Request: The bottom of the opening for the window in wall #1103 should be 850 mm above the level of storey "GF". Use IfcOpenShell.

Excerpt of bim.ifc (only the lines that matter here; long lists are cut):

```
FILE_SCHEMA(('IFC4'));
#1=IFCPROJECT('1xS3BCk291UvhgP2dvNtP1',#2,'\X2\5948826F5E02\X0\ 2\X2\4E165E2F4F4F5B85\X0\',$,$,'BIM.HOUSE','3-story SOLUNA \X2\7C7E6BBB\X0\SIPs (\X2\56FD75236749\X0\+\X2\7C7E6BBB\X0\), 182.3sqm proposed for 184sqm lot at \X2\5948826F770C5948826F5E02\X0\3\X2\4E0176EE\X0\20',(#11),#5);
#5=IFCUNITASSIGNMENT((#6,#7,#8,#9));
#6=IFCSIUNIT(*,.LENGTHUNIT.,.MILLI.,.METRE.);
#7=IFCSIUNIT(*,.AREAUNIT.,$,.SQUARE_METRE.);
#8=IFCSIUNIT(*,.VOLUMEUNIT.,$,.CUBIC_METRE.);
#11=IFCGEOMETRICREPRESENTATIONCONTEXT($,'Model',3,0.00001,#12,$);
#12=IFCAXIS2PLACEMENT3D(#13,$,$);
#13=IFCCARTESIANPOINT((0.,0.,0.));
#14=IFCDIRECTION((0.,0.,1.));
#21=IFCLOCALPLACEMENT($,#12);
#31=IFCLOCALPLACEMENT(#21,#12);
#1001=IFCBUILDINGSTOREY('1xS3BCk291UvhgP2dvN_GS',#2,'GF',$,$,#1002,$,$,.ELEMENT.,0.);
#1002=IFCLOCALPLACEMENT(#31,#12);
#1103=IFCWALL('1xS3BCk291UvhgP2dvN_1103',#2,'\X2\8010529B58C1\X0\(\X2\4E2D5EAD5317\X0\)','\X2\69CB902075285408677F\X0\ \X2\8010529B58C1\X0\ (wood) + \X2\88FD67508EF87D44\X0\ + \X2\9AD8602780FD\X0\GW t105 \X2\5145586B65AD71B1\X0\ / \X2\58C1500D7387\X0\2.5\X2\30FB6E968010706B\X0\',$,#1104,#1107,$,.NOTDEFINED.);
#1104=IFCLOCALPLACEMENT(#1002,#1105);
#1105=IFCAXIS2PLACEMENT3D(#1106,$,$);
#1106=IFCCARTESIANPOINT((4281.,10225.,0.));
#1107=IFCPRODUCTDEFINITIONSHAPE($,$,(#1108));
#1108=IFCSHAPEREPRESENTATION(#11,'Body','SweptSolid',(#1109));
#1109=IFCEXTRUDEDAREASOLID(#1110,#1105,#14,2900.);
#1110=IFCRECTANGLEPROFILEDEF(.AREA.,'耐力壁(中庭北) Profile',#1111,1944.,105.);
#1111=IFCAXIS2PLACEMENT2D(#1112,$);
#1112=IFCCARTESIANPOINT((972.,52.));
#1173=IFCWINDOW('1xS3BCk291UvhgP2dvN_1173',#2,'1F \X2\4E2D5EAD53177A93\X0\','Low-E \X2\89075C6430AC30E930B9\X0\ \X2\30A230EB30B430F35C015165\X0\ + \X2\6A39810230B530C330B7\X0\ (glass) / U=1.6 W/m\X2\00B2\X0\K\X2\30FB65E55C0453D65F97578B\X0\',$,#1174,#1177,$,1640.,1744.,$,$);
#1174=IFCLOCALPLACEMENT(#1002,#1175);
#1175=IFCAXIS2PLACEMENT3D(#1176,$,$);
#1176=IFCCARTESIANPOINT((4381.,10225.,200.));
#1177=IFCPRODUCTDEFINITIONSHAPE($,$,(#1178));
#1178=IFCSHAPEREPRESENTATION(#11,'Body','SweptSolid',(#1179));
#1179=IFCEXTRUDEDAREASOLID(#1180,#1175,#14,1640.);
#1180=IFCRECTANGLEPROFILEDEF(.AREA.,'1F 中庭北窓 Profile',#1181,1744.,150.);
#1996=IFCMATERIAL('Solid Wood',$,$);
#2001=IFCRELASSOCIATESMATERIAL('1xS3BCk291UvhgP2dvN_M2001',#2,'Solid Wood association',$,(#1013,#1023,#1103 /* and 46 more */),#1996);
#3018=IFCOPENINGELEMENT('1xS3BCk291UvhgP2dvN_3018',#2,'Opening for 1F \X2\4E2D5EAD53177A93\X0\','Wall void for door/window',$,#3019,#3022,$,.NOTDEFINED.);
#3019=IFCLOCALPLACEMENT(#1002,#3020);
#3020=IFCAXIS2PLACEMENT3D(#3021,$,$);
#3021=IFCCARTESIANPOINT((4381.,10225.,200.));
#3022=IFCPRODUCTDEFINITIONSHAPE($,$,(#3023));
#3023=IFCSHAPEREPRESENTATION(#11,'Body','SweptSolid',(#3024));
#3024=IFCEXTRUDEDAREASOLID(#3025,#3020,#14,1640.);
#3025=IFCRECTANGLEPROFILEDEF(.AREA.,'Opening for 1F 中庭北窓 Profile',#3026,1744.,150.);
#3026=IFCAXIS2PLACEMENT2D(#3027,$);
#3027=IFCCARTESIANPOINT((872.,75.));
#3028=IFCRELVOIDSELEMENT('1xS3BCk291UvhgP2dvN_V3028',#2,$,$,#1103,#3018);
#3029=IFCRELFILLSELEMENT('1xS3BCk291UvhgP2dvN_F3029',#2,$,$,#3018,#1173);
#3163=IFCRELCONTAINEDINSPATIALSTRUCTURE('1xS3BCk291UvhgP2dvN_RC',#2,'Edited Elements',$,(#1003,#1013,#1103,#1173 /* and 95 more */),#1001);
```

```python
import numpy as np
import ifcopenshell
import ifcopenshell.api.geometry
import ifcopenshell.geom
import ifcopenshell.util.element
import ifcopenshell.util.placement
import ifcopenshell.util.shape
import ifcopenshell.util.unit

model = ifcopenshell.open("bim.ifc")
unit_scale = ifcopenshell.util.unit.calculate_unit_scale(model)

window = model.by_id(1173)
opening = window.FillsVoids[0].RelatingOpeningElement
storey = ifcopenshell.util.element.get_container(window, ifc_class="IfcBuildingStorey")
level = ifcopenshell.util.placement.get_local_placement(storey.ObjectPlacement)[2, 3]

# The opening's origin need not be at the sill, so measure its lowest point.
shape = ifcopenshell.geom.create_shape(ifcopenshell.geom.settings(), opening)
bottom = ifcopenshell.util.shape.get_shape_bottom_elevation(shape, shape.geometry) / unit_scale
dz = level + 850.0 - bottom

shift = np.array([0.0, 0.0, dz])
# The window is not placed relative to its opening, so move both.
for product in (opening, window):
    matrix = ifcopenshell.util.placement.get_local_placement(product.ObjectPlacement)
    matrix[:3, 3] += shift
    ifcopenshell.api.geometry.edit_object_placement(model, product=product, matrix=matrix, is_si=False)

print(f"moved by {dz * unit_scale:+.3f} m")

model.write("bim_edited.ifc")
```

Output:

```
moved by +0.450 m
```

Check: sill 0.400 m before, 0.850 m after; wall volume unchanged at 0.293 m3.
